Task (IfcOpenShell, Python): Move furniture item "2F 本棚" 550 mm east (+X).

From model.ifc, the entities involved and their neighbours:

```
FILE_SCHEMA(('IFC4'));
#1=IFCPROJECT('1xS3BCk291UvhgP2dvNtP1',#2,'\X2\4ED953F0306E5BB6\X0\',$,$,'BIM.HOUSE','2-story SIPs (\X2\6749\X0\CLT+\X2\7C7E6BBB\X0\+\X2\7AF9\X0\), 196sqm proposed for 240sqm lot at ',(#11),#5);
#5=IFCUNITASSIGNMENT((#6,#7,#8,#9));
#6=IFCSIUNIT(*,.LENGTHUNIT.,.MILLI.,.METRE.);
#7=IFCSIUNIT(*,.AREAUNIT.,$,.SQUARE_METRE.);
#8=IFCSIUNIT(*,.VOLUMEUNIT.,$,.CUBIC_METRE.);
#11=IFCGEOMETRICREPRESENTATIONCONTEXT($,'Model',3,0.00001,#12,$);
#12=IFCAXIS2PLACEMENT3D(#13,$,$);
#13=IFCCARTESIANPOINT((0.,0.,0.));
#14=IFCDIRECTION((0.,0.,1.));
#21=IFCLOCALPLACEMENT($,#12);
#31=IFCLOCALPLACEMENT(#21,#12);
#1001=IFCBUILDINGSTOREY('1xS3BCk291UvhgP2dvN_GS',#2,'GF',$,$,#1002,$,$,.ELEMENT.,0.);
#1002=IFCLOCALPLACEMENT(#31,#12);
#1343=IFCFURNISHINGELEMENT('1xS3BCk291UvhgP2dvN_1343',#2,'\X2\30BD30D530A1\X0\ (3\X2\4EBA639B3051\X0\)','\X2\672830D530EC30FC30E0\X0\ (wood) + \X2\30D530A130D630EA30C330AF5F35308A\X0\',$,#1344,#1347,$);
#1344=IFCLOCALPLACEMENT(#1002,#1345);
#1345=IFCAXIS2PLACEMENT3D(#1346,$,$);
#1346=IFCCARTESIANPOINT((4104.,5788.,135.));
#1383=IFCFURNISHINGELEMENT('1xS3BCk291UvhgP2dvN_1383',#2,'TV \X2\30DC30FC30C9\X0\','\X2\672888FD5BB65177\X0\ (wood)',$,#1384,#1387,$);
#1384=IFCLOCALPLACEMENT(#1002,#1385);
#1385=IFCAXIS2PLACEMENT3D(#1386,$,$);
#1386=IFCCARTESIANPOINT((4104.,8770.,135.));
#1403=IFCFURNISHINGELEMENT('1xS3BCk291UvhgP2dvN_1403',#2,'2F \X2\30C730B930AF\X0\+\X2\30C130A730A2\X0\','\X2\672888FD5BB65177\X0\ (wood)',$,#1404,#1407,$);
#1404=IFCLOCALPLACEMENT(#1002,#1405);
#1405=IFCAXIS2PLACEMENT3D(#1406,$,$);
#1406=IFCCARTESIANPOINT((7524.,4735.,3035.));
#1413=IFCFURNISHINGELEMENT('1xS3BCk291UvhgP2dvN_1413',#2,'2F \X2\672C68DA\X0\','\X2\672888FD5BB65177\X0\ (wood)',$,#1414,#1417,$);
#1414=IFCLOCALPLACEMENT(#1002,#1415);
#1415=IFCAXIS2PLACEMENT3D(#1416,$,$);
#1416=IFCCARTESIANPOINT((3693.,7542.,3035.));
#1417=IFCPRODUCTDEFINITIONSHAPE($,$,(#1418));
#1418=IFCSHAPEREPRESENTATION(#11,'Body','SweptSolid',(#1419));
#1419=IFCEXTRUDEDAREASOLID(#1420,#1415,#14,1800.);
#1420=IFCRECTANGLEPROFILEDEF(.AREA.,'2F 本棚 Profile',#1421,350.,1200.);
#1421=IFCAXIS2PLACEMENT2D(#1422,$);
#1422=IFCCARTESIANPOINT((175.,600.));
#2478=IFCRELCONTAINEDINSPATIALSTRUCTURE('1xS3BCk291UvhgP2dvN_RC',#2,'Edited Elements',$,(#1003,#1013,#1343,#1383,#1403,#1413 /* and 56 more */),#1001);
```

```python
import ifcopenshell
import ifcopenshell.api.geometry
import ifcopenshell.util.placement

model = ifcopenshell.open("model.ifc")

item = model.by_guid("1xS3BCk291UvhgP2dvN_1413")
matrix = ifcopenshell.util.placement.get_local_placement(item.ObjectPlacement)
matrix[0, 3] += 550.0
ifcopenshell.api.geometry.edit_object_placement(model, product=item, matrix=matrix, is_si=False)

print(ifcopenshell.util.placement.get_local_placement(item.ObjectPlacement).round(3) + 0.0)

model.write("model_v2.ifc")
```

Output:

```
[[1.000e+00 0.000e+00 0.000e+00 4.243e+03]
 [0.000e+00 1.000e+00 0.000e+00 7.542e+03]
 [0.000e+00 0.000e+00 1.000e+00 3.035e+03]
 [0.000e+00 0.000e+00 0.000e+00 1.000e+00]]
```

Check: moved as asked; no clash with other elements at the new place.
